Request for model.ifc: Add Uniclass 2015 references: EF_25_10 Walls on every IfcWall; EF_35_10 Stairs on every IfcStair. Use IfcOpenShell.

First a look at what the model holds.

```python
import ifcopenshell

model = ifcopenshell.open("model.ifc")
print(model.schema)
print("classifications:", [c.Name for c in model.by_type("IfcClassification")])
for ifc_class in ("IfcDoor", "IfcRoof", "IfcStair", "IfcWall", "IfcWindow"):
    print(ifc_class, len(model.by_type(ifc_class)))
```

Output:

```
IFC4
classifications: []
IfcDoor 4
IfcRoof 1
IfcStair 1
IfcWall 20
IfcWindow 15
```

```python
import ifcopenshell
import ifcopenshell.api.classification

model = ifcopenshell.open("model.ifc")

system = ifcopenshell.api.classification.add_classification(model, classification="Uniclass 2015")

codes = {
    "IfcWall": ("EF_25_10", "Walls"),
    "IfcStair": ("EF_35_10", "Stairs"),
}
for ifc_class, (code, name) in codes.items():
    products = model.by_type(ifc_class)
    ifcopenshell.api.classification.add_reference(
        model, products=products, classification=system, identification=code, name=name
    )
    print(code, len(products))

model.write("model-out.ifc")
```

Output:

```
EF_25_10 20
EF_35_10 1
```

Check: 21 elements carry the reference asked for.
